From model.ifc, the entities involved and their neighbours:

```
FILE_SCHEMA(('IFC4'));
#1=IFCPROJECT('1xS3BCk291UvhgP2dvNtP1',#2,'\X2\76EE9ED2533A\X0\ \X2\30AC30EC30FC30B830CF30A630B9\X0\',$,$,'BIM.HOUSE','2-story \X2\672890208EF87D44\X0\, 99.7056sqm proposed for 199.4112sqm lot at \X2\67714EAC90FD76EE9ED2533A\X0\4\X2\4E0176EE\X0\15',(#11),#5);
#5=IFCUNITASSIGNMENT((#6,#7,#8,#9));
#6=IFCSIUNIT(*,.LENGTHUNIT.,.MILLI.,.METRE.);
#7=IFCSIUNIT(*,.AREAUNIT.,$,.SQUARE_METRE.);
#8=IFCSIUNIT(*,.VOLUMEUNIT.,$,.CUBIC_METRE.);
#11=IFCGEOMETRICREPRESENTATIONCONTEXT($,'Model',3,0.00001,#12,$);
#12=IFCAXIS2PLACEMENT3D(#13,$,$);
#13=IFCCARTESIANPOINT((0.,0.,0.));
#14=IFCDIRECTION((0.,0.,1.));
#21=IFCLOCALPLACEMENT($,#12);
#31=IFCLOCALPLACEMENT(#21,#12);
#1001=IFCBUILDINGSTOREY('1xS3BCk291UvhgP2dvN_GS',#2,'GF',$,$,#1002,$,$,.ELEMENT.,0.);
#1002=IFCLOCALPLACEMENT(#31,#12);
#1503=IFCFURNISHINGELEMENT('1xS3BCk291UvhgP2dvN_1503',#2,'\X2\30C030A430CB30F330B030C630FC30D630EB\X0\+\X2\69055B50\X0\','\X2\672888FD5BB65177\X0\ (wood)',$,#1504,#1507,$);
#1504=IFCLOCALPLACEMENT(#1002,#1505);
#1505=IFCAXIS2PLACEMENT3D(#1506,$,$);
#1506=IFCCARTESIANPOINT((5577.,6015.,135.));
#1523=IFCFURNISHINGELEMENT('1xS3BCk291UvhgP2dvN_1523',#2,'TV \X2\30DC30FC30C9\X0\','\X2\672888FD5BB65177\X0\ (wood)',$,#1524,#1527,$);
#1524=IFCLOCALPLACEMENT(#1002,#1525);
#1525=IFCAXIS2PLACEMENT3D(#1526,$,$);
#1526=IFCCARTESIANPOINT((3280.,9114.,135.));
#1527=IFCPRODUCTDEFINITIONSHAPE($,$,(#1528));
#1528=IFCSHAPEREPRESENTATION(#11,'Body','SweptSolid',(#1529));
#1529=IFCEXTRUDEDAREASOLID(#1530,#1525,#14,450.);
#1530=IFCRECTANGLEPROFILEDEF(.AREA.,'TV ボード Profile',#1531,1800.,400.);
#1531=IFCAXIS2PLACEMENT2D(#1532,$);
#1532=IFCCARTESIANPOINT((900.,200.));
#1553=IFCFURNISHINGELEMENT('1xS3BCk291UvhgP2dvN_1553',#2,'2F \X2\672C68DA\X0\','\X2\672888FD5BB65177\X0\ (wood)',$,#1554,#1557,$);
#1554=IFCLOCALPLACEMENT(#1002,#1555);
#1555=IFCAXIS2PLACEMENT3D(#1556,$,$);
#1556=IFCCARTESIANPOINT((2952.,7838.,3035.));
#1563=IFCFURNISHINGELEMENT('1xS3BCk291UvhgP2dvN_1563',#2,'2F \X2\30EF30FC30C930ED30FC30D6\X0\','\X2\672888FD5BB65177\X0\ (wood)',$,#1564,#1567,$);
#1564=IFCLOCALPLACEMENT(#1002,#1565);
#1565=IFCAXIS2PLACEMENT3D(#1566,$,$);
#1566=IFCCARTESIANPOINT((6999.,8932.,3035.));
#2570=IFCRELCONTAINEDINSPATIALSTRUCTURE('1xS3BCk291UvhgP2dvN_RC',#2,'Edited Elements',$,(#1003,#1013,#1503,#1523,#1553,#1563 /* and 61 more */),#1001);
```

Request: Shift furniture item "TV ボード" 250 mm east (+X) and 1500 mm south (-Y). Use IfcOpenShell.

```python
import ifcopenshell
import ifcopenshell.api.geometry
import ifcopenshell.util.placement
import ifcopenshell.util.unit

model = ifcopenshell.open("model.ifc")
unit_scale = ifcopenshell.util.unit.calculate_unit_scale(model)

item = model.by_guid("1xS3BCk291UvhgP2dvN_1523")
matrix = ifcopenshell.util.placement.get_local_placement(item.ObjectPlacement)
matrix[0, 3] += 0.25 / unit_scale
matrix[1, 3] -= 1.5 / unit_scale
ifcopenshell.api.geometry.edit_object_placement(model, product=item, matrix=matrix, is_si=False)

print(ifcopenshell.util.placement.get_local_placement(item.ObjectPlacement).round(3) + 0.0)

model.write("model_v2.ifc")
```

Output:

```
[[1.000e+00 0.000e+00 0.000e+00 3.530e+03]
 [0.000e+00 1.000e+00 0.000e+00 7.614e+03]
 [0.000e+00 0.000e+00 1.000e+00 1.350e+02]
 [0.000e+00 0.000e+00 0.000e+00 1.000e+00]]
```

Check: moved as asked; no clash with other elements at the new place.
